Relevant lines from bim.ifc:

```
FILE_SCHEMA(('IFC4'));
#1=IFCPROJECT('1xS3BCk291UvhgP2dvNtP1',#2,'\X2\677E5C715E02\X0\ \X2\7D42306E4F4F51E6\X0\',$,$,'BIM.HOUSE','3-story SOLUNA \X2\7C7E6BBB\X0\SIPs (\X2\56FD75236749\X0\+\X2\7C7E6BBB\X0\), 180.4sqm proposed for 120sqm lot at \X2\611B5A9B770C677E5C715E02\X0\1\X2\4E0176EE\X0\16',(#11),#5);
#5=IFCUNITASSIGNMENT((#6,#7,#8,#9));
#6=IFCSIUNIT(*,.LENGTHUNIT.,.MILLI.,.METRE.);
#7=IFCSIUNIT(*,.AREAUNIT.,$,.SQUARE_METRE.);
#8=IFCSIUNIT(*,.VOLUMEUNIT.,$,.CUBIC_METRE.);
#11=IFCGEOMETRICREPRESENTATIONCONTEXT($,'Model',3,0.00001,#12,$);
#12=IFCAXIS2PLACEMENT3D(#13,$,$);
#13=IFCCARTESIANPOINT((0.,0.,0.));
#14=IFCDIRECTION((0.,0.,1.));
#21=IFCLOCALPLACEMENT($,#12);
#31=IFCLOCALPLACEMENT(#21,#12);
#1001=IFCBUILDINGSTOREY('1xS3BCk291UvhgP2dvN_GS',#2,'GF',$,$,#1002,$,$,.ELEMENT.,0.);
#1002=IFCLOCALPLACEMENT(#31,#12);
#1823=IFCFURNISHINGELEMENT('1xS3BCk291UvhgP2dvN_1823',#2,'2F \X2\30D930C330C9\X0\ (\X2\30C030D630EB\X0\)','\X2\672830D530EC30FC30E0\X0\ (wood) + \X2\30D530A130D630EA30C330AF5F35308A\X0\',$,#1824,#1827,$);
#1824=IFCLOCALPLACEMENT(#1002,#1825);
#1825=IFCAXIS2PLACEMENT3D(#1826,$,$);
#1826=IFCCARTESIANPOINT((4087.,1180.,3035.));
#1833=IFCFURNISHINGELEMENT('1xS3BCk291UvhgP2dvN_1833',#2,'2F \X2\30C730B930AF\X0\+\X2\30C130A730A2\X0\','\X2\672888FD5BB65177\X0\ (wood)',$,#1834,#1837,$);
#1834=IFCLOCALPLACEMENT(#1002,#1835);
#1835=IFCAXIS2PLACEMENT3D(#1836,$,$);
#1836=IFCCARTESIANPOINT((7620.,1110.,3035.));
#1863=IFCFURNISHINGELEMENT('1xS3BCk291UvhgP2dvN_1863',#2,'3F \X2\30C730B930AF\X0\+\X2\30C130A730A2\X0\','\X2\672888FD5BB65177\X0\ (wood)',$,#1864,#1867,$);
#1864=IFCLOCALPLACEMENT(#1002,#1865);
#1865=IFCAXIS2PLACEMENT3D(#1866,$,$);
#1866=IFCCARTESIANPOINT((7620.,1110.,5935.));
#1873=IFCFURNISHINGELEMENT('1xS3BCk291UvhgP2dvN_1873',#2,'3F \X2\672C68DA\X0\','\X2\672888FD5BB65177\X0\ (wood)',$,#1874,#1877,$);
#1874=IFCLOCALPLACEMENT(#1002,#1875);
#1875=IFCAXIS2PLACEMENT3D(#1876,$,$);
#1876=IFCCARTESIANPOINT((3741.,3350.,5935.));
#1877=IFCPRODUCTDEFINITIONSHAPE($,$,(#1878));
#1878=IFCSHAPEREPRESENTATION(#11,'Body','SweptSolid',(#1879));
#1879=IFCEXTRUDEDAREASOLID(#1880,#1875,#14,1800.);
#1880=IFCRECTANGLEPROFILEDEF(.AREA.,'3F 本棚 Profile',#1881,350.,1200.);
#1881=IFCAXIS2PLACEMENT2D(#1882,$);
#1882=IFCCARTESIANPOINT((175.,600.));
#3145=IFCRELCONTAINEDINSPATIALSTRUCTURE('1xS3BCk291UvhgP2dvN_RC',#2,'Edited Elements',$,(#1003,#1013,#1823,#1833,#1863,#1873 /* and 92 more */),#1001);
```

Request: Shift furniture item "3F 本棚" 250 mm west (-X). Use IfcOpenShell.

```python
import ifcopenshell
import ifcopenshell.api.geometry
import ifcopenshell.util.placement
import ifcopenshell.util.unit

model = ifcopenshell.open("bim.ifc")
unit_scale = ifcopenshell.util.unit.calculate_unit_scale(model)

item = model.by_id(1873)
matrix = ifcopenshell.util.placement.get_local_placement(item.ObjectPlacement)
matrix[0, 3] -= 0.25 / unit_scale
ifcopenshell.api.geometry.edit_object_placement(model, product=item, matrix=matrix, is_si=False)

print(ifcopenshell.util.placement.get_local_placement(item.ObjectPlacement).round(3) + 0.0)

model.write("bim_updated.ifc")
```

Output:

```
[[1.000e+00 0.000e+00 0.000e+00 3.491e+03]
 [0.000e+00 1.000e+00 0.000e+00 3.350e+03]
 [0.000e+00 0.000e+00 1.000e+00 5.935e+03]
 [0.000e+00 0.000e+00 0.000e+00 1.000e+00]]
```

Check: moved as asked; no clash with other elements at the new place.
